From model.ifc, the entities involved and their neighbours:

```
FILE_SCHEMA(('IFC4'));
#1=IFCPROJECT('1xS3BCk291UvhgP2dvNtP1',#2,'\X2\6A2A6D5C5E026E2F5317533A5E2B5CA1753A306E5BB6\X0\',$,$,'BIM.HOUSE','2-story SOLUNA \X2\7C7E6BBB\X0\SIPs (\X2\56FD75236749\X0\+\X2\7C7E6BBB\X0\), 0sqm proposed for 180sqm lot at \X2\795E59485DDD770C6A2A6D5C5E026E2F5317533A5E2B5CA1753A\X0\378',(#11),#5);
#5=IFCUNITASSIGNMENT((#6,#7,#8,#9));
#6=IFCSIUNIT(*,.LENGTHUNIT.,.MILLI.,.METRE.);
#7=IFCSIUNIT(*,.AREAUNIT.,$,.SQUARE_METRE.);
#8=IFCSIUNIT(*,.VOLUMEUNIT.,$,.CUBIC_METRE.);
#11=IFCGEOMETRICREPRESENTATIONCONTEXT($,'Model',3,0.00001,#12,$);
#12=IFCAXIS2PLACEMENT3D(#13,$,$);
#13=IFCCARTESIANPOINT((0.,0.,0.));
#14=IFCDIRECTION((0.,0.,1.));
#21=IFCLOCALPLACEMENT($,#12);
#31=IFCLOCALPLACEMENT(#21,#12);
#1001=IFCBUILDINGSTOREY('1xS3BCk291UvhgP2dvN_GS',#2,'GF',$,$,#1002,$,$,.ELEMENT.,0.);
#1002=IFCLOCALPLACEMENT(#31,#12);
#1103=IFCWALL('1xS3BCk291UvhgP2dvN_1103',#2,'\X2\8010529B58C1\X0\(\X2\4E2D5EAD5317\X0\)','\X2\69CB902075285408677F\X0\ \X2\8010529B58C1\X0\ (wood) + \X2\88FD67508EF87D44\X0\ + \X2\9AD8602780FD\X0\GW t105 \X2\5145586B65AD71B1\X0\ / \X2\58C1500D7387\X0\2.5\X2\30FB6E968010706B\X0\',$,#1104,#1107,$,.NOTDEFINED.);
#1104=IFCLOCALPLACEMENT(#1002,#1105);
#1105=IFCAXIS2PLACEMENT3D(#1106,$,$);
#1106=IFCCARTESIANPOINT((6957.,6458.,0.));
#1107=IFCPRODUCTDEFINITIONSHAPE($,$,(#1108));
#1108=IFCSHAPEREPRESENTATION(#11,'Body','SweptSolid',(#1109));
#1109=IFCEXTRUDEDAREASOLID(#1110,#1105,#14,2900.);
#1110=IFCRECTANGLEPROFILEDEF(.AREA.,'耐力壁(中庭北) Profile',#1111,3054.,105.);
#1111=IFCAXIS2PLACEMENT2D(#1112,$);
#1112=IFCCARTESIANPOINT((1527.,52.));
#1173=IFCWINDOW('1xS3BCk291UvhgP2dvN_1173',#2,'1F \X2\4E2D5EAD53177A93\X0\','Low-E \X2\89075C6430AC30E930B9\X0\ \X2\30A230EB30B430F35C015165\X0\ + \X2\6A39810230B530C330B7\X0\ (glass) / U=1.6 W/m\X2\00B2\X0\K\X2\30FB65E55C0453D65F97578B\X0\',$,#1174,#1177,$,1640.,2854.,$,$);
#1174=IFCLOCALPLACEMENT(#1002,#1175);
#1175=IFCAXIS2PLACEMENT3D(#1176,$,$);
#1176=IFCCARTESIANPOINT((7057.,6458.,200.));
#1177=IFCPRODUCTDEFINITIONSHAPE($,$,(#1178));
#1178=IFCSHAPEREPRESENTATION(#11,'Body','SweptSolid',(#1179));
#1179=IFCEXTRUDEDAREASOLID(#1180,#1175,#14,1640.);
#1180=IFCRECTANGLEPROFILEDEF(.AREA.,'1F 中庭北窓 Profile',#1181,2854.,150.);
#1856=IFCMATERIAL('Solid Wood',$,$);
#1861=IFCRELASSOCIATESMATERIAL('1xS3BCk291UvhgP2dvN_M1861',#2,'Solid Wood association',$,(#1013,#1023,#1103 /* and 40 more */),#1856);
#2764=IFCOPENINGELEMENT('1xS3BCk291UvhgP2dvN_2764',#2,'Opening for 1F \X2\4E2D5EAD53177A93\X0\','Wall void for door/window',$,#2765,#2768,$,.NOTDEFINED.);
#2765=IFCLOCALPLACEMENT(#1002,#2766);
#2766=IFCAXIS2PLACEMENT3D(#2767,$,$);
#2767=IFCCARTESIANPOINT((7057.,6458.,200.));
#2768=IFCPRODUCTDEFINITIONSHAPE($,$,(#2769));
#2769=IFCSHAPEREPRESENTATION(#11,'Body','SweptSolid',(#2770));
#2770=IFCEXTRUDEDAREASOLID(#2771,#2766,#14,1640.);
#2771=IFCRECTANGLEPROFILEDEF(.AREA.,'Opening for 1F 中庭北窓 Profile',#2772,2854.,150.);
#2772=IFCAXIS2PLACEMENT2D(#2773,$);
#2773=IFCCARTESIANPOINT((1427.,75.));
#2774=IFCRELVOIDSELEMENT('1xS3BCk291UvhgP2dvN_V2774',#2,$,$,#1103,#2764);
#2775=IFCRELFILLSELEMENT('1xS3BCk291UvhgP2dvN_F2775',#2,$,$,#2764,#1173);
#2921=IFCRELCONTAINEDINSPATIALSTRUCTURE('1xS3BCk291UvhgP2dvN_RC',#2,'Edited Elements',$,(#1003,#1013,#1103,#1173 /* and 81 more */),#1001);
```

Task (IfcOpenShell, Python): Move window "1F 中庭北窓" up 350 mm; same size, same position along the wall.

```python
import numpy as np
import ifcopenshell
import ifcopenshell.api.geometry
import ifcopenshell.util.placement
import ifcopenshell.util.unit

model = ifcopenshell.open("model.ifc")
unit_scale = ifcopenshell.util.unit.calculate_unit_scale(model)

window = model.by_id(1173)
opening = window.FillsVoids[0].RelatingOpeningElement
dz = 350.0

shift = np.array([0.0, 0.0, dz])
# The window is not placed relative to its opening, so move both.
for product in (opening, window):
    matrix = ifcopenshell.util.placement.get_local_placement(product.ObjectPlacement)
    matrix[:3, 3] += shift
    ifcopenshell.api.geometry.edit_object_placement(model, product=product, matrix=matrix, is_si=False)

print(f"moved by {dz * unit_scale:+.3f} m")

model.write("model_rev.ifc")
```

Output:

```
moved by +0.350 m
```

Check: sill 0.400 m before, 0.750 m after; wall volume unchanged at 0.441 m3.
